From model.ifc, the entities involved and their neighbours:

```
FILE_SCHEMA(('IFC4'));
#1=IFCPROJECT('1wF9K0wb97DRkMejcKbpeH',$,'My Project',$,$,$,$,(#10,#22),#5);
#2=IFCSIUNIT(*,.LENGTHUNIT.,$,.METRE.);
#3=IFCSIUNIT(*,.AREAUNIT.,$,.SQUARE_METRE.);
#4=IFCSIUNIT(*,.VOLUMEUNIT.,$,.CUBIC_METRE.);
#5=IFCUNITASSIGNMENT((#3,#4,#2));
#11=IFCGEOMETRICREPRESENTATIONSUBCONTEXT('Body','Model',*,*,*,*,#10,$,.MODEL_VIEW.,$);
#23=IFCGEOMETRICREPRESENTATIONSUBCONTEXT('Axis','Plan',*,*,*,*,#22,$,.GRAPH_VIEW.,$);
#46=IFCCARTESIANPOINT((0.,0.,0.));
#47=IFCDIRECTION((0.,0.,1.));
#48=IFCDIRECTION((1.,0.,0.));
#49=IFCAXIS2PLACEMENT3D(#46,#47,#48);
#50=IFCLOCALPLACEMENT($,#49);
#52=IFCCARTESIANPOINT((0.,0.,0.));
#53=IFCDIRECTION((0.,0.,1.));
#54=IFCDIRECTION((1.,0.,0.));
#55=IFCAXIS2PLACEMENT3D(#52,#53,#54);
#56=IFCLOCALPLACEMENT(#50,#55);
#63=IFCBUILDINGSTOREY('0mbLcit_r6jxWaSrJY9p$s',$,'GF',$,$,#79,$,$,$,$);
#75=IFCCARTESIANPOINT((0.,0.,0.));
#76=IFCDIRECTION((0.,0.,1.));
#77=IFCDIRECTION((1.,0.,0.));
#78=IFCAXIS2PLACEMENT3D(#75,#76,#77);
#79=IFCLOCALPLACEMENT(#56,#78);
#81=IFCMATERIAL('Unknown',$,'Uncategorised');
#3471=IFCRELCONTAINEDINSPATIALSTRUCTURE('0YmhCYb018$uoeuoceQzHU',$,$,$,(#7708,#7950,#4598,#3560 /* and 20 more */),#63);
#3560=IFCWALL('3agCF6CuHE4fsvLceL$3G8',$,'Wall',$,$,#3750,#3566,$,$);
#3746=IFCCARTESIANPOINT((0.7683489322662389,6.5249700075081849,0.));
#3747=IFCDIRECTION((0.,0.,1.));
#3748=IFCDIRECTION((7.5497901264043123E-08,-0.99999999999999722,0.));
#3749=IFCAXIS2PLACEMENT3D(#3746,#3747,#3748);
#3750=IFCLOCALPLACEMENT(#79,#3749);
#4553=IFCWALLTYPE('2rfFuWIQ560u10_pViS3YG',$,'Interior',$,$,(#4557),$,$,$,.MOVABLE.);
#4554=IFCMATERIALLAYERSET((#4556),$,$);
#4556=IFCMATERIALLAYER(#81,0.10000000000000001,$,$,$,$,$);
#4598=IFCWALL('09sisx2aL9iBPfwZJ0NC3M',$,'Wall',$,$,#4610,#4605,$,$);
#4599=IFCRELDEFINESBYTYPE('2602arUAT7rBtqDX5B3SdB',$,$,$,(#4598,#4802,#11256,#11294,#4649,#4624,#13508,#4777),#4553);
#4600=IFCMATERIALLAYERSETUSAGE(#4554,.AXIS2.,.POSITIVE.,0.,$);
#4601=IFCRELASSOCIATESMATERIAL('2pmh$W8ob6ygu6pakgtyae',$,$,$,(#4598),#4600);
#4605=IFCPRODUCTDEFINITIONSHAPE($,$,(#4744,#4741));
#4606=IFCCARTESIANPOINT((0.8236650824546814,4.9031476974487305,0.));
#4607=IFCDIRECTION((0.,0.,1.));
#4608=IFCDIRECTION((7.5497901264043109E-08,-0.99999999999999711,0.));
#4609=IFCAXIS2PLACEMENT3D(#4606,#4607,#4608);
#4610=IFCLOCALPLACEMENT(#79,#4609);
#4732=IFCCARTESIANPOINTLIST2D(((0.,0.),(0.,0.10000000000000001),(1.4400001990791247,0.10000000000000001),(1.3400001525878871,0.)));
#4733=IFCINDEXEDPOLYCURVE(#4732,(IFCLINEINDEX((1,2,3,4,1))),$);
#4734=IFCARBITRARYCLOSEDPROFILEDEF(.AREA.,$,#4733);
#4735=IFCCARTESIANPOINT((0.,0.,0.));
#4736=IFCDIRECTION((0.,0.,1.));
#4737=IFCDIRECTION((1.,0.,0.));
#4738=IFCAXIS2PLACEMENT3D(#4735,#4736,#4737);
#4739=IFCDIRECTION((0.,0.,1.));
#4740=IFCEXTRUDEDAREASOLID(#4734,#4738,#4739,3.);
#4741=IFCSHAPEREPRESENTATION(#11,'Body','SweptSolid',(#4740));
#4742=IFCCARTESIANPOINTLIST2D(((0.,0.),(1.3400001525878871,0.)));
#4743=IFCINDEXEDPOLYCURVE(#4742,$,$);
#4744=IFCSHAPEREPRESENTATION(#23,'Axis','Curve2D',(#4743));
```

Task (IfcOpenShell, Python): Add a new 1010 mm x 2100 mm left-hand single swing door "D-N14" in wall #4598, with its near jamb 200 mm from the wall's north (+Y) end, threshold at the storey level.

```python
import numpy as np
import ifcopenshell
import ifcopenshell.api.feature
import ifcopenshell.api.geometry
import ifcopenshell.api.root
import ifcopenshell.api.spatial
import ifcopenshell.geom
import ifcopenshell.util.element
import ifcopenshell.util.placement
import ifcopenshell.util.representation
import ifcopenshell.util.shape
import ifcopenshell.util.unit

model = ifcopenshell.open("model.ifc")
unit_scale = ifcopenshell.util.unit.calculate_unit_scale(model)
settings = ifcopenshell.geom.settings()


def volume(element):
    """Net volume in cubic metres, openings subtracted."""
    shape = ifcopenshell.geom.create_shape(settings, element)
    return ifcopenshell.util.shape.get_volume(shape.geometry)


wall = model.by_id(4598)
storey = ifcopenshell.util.element.get_container(wall, ifc_class="IfcBuildingStorey")
context = ifcopenshell.util.representation.get_context(model, "Model", "Body", "MODEL_VIEW")
before = volume(wall)

width, height, from_end, sill = 1.01, 2.1, 0.2, 0.0  # metres

# The wall runs along its own X axis, and the end named is its -X end.
wall_shape = ifcopenshell.geom.create_shape(settings, wall)
x, y, z = ifcopenshell.util.shape.get_vertices(wall_shape.geometry).T
start = x.min() + from_end
face, thickness = float(y.min()), float(y.max() - y.min())
wall_matrix = ifcopenshell.util.placement.get_local_placement(wall.ObjectPlacement)
level = ifcopenshell.util.placement.get_local_placement(storey.ObjectPlacement)[2, 3]


def in_wall(x, y):
    """Placement at x, y metres in the wall's axes, at sill height."""
    matrix = wall_matrix.copy()
    matrix[:, 3] = wall_matrix @ np.array([x / unit_scale, y / unit_scale, 0.0, 1.0])
    matrix[2, 3] = level + sill / unit_scale
    return matrix


# Opening: a box that overshoots both wall faces by 50 mm.
opening = ifcopenshell.api.root.create_entity(model, ifc_class="IfcOpeningElement", predefined_type="OPENING")
box = ifcopenshell.api.geometry.add_wall_representation(
    model, context=context, length=width, height=height, thickness=thickness + 0.1
)
ifcopenshell.api.geometry.assign_representation(model, product=opening, representation=box)
ifcopenshell.api.geometry.edit_object_placement(model, product=opening, matrix=in_wall(start, face - 0.05), is_si=False)
ifcopenshell.api.feature.add_feature(model, feature=opening, element=wall)

door = ifcopenshell.api.root.create_entity(model, ifc_class="IfcDoor", name="D-N14", predefined_type="DOOR")
door.OverallWidth, door.OverallHeight = width / unit_scale, height / unit_scale
door.OperationType = "SINGLE_SWING_LEFT"
body = ifcopenshell.api.geometry.add_door_representation(
    model,
    context=context,
    overall_width=door.OverallWidth,
    overall_height=door.OverallHeight,
    operation_type="SINGLE_SWING_LEFT",
    lining_properties={"LiningDepth": thickness / unit_scale, "ThresholdDepth": thickness / unit_scale},
)
ifcopenshell.api.geometry.assign_representation(model, product=door, representation=body)
ifcopenshell.api.spatial.assign_container(model, products=[door], relating_structure=storey)
ifcopenshell.api.feature.add_filling(model, opening=opening, element=door)

# The lining spans the wall, so the door starts at the wall face.
ifcopenshell.api.geometry.edit_object_placement(model, product=door, matrix=in_wall(start, face), is_si=False)

after = volume(wall)

print(f"wall volume {before:.3f} -> {after:.3f} m3")

model.write("model_rev.ifc")
```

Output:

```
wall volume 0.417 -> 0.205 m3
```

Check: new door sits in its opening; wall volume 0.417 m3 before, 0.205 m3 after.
